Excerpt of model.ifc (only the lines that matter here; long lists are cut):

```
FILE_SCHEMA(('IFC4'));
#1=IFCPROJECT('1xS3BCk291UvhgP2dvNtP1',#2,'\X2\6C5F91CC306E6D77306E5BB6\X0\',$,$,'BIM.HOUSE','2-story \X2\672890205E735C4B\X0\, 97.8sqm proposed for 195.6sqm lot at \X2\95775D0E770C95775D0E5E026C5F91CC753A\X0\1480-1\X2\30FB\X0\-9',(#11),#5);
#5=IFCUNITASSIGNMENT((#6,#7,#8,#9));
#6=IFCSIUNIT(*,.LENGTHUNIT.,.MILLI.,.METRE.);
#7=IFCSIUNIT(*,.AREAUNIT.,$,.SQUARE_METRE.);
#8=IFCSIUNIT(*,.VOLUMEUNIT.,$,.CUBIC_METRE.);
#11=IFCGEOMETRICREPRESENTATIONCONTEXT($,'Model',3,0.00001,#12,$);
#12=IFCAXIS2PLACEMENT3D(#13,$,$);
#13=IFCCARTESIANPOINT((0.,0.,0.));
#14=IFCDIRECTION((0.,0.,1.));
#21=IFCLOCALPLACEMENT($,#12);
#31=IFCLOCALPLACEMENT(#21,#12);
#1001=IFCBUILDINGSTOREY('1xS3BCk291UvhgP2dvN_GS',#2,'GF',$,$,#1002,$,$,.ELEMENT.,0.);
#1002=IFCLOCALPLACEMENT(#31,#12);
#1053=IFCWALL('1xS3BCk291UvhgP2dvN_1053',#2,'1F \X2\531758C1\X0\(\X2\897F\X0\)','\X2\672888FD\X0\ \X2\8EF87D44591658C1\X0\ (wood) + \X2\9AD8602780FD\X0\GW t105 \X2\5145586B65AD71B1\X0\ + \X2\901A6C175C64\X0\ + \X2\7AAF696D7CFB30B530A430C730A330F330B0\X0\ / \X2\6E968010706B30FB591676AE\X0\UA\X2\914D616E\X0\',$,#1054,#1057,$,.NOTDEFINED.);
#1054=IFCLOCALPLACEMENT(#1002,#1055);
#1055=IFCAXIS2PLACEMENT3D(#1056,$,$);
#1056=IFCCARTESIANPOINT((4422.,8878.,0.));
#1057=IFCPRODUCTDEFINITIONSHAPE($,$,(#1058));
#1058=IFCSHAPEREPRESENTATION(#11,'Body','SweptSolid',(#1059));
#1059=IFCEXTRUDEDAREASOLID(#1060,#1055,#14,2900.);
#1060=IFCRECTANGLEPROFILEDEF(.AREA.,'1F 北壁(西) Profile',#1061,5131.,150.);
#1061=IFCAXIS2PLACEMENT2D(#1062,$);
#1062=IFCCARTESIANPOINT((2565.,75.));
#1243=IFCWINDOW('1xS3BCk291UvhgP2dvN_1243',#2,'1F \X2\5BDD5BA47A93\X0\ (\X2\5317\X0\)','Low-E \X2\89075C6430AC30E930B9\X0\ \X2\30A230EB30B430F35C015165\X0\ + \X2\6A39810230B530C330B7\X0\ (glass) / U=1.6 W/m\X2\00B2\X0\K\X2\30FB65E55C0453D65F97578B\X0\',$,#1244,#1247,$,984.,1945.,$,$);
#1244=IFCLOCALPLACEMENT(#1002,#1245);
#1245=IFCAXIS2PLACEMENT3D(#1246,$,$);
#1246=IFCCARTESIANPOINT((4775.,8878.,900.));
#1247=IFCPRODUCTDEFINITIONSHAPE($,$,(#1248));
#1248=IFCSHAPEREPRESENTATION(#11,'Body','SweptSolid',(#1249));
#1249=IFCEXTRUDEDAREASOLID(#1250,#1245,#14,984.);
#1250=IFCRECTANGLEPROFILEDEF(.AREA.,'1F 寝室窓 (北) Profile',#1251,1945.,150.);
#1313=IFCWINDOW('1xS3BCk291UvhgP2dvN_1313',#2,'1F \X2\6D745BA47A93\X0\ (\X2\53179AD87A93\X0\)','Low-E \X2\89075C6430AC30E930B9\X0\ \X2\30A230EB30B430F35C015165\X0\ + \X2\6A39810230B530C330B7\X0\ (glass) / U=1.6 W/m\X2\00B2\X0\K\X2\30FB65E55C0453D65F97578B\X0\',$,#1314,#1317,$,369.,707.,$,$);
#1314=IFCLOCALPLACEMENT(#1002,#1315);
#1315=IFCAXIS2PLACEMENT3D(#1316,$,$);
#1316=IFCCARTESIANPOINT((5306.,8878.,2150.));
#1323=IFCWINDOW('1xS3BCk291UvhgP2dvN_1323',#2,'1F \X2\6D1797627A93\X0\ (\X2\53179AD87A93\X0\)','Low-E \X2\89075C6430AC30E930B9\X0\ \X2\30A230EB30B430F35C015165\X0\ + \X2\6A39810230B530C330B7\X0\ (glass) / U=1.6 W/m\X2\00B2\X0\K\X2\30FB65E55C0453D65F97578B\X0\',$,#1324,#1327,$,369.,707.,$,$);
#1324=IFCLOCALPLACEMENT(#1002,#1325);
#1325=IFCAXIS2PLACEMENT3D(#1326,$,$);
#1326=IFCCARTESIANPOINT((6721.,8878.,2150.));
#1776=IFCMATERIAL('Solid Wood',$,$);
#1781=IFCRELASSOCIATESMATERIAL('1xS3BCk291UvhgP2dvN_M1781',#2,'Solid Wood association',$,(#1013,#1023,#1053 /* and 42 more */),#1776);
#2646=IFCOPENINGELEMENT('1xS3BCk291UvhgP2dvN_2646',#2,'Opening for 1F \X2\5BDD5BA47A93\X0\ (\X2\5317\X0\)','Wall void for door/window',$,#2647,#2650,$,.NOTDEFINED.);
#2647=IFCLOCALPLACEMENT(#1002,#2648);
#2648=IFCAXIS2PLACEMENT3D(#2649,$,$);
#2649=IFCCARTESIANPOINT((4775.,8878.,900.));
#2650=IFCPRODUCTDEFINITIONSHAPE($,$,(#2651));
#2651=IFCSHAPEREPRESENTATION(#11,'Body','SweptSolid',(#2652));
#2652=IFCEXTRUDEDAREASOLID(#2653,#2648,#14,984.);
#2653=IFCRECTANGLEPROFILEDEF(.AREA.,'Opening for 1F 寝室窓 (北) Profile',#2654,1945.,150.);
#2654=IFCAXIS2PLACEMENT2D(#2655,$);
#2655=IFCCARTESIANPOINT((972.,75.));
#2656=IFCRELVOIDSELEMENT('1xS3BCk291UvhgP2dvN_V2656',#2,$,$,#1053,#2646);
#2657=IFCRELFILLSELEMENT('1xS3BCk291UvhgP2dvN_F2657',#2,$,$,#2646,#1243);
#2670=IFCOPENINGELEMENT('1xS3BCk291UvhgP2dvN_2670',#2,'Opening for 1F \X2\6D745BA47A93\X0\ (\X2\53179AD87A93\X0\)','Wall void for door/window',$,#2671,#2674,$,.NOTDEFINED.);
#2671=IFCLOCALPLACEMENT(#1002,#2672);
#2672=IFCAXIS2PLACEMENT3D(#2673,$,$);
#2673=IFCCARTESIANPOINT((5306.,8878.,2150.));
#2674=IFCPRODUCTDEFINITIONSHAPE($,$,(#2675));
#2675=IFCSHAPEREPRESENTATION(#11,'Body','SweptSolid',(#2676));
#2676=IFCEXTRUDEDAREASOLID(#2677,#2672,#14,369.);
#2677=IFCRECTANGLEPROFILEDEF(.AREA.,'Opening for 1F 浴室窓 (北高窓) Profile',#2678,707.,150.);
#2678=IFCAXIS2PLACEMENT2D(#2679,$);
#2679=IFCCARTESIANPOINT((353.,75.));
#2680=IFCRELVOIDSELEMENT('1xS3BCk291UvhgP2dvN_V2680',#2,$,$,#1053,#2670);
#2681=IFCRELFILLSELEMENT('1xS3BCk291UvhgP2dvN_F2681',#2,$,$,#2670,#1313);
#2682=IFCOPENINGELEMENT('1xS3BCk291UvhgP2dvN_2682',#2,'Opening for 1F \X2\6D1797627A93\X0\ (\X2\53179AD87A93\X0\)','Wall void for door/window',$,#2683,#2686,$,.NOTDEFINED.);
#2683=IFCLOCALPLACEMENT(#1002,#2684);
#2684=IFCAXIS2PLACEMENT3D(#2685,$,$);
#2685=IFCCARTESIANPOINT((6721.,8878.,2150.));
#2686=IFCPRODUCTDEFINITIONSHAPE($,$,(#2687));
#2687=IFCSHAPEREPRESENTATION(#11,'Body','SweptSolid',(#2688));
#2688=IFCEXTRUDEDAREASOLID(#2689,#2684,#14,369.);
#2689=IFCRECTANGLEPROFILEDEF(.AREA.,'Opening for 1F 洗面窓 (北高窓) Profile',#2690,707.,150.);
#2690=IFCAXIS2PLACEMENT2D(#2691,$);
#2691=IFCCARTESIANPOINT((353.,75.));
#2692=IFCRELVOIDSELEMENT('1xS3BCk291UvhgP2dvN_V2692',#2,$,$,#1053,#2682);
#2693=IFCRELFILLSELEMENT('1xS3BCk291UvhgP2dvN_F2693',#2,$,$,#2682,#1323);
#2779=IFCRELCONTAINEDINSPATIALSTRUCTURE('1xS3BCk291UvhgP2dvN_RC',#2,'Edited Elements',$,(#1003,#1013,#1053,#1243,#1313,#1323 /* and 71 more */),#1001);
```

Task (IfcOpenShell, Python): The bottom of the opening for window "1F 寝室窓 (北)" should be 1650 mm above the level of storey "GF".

```python
import numpy as np
import ifcopenshell
import ifcopenshell.api.geometry
import ifcopenshell.geom
import ifcopenshell.util.element
import ifcopenshell.util.placement
import ifcopenshell.util.shape
import ifcopenshell.util.unit

model = ifcopenshell.open("model.ifc")
unit_scale = ifcopenshell.util.unit.calculate_unit_scale(model)

window = model.by_guid("1xS3BCk291UvhgP2dvN_1243")
opening = window.FillsVoids[0].RelatingOpeningElement
storey = ifcopenshell.util.element.get_container(window, ifc_class="IfcBuildingStorey")
level = ifcopenshell.util.placement.get_local_placement(storey.ObjectPlacement)[2, 3]

# The opening's origin need not be at the sill, so measure its lowest point.
shape = ifcopenshell.geom.create_shape(ifcopenshell.geom.settings(), opening)
bottom = ifcopenshell.util.shape.get_shape_bottom_elevation(shape, shape.geometry) / unit_scale
dz = level + 1650.0 - bottom

shift = np.array([0.0, 0.0, dz])
# The window is not placed relative to its opening, so move both.
for product in (opening, window):
    matrix = ifcopenshell.util.placement.get_local_placement(product.ObjectPlacement)
    matrix[:3, 3] += shift
    ifcopenshell.api.geometry.edit_object_placement(model, product=product, matrix=matrix, is_si=False)

print(f"moved by {dz * unit_scale:+.3f} m")

model.write("model_v2.ifc")
```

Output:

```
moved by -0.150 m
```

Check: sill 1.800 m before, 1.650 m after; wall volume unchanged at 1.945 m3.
